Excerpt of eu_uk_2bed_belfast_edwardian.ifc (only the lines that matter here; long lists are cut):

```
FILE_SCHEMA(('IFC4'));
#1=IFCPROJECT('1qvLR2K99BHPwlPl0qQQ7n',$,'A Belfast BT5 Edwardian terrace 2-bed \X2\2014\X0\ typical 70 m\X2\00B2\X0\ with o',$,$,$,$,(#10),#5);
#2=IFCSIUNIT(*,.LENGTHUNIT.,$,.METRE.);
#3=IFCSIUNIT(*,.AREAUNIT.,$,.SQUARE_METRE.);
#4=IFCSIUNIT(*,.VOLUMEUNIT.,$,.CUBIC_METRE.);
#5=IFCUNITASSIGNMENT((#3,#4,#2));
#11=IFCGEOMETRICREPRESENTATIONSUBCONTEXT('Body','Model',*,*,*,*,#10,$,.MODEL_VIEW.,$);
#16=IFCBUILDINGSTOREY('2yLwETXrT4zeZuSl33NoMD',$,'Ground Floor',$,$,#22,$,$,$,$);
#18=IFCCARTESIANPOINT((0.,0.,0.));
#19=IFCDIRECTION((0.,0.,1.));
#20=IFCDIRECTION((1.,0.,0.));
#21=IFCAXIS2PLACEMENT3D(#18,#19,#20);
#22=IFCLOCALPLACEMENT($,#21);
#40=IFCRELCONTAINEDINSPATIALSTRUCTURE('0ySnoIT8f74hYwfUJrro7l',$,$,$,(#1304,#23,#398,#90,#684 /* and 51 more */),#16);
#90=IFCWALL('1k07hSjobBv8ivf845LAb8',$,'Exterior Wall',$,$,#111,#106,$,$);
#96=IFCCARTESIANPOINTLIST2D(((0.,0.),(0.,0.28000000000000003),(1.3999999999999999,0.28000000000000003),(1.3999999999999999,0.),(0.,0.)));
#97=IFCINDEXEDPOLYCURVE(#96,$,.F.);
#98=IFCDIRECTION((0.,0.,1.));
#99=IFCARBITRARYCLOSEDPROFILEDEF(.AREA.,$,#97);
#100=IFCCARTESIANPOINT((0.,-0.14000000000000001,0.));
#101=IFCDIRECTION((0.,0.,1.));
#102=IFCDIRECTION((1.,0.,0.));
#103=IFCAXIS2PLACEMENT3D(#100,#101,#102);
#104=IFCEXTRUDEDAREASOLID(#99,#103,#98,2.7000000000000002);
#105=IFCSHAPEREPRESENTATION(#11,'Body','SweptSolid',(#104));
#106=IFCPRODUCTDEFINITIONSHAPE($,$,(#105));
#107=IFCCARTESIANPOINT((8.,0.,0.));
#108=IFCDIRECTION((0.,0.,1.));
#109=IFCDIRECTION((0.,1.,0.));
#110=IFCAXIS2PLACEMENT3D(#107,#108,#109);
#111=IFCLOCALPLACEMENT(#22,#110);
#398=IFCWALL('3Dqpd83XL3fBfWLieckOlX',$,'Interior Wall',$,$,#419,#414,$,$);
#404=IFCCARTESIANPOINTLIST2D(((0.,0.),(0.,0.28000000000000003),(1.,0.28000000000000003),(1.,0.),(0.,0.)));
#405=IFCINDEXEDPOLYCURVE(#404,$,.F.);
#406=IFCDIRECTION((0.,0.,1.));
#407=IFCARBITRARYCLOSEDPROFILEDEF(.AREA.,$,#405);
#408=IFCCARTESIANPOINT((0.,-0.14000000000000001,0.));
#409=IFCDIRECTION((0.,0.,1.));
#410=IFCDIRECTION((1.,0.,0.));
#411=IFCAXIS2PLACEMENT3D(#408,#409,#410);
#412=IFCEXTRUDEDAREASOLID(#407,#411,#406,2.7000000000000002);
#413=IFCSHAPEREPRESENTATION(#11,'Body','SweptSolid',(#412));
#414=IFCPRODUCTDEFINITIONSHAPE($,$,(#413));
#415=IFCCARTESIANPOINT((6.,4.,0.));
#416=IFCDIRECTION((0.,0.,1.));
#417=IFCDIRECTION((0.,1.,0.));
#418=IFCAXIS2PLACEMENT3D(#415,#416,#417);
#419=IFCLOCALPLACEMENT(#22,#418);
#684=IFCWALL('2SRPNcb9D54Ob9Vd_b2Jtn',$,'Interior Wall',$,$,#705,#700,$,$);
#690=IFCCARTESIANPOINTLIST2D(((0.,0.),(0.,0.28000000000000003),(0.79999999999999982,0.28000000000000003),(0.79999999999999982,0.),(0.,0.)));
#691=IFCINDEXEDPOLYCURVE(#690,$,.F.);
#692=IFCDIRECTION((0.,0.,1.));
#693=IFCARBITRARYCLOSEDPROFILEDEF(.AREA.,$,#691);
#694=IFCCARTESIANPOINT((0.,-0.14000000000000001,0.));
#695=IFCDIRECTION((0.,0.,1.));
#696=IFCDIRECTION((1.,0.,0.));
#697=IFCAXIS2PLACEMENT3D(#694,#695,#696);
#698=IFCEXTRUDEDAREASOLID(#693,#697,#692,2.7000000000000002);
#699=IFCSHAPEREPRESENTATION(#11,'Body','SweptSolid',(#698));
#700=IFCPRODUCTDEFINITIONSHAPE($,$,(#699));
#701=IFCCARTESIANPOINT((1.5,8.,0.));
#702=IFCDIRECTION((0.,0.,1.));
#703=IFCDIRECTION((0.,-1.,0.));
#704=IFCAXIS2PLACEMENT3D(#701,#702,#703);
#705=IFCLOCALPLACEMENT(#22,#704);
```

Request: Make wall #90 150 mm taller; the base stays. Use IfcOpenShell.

```python
import ifcopenshell
import ifcopenshell.geom
import ifcopenshell.util.representation
import ifcopenshell.util.shape
import ifcopenshell.util.unit

model = ifcopenshell.open("eu_uk_2bed_belfast_edwardian.ifc")
unit_scale = ifcopenshell.util.unit.calculate_unit_scale(model)
settings = ifcopenshell.geom.settings()


def volume(element):
    """Net volume in cubic metres, openings subtracted."""
    shape = ifcopenshell.geom.create_shape(settings, element)
    return ifcopenshell.util.shape.get_volume(shape.geometry)


wall = model.by_guid("1k07hSjobBv8ivf845LAb8")
before = volume(wall)

body = ifcopenshell.util.representation.get_representation(wall, "Model", "Body")
solid = body.Items[0]
old_height = solid.Depth
solid.Depth += 0.15 / unit_scale
after = volume(wall)

print(f"height {old_height:g} -> {solid.Depth:g}, volume {before:.3f} -> {after:.3f} m3")

model.write("eu_uk_2bed_belfast_edwardian_rev.ifc")
```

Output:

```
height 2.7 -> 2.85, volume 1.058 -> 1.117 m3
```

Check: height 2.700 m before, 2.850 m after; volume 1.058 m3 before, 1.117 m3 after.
